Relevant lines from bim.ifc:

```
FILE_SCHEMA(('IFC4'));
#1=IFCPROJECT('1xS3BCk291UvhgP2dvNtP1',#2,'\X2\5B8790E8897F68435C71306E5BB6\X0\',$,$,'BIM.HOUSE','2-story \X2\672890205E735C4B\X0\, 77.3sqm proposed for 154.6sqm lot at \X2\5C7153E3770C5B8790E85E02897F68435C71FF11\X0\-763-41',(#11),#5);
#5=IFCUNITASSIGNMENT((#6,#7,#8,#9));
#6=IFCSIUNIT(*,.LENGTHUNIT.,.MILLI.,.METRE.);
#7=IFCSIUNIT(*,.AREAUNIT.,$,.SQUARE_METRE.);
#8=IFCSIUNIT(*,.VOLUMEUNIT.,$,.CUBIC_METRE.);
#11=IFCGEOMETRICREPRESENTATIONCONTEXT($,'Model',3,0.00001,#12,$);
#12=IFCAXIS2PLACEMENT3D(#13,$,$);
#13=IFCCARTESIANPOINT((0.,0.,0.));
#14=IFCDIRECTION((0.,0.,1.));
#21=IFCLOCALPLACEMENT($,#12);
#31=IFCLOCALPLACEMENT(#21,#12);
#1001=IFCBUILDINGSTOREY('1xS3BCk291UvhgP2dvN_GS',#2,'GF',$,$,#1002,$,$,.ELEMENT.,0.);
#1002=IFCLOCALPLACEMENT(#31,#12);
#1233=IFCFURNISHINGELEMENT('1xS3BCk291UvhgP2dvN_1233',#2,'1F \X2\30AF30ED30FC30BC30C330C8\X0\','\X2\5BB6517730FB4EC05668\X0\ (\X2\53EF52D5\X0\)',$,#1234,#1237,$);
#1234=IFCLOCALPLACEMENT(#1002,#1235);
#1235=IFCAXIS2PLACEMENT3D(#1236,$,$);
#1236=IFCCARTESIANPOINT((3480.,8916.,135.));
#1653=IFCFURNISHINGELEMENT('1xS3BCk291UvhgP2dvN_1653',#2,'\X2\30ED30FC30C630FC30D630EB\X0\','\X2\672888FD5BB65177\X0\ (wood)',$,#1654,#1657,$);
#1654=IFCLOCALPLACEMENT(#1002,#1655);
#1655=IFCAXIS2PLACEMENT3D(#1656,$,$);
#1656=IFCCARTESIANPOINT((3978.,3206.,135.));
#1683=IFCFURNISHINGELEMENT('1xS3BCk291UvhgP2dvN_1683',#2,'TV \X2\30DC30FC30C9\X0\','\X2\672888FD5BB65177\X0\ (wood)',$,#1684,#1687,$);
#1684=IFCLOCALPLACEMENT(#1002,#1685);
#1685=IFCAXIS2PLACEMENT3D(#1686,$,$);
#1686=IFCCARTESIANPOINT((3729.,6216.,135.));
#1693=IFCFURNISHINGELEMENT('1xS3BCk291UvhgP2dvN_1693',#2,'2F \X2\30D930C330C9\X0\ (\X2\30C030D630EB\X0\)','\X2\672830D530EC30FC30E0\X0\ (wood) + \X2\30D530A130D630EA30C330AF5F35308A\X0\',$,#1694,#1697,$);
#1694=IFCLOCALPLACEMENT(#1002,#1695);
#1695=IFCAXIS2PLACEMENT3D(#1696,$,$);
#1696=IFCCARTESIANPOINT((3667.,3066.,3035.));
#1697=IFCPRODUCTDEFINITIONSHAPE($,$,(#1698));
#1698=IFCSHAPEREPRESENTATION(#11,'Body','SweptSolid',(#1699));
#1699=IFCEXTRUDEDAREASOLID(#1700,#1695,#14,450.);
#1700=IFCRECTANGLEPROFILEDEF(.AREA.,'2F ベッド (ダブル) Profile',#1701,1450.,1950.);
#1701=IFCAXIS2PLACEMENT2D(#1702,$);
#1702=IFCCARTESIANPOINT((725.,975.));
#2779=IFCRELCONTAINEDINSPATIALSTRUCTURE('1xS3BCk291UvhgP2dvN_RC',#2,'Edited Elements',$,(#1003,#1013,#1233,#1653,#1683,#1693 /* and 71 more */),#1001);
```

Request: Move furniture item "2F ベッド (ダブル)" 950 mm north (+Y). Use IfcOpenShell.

```python
import ifcopenshell
import ifcopenshell.api.geometry
import ifcopenshell.util.placement

model = ifcopenshell.open("bim.ifc")

item = model.by_guid("1xS3BCk291UvhgP2dvN_1693")
matrix = ifcopenshell.util.placement.get_local_placement(item.ObjectPlacement)
matrix[1, 3] += 950.0
ifcopenshell.api.geometry.edit_object_placement(model, product=item, matrix=matrix, is_si=False)

print(ifcopenshell.util.placement.get_local_placement(item.ObjectPlacement).round(3) + 0.0)

model.write("bim_rev.ifc")
```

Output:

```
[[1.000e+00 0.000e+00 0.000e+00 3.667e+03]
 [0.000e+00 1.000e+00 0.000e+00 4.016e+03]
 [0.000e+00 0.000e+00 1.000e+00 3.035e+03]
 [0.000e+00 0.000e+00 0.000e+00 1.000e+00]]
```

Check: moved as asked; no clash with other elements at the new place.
